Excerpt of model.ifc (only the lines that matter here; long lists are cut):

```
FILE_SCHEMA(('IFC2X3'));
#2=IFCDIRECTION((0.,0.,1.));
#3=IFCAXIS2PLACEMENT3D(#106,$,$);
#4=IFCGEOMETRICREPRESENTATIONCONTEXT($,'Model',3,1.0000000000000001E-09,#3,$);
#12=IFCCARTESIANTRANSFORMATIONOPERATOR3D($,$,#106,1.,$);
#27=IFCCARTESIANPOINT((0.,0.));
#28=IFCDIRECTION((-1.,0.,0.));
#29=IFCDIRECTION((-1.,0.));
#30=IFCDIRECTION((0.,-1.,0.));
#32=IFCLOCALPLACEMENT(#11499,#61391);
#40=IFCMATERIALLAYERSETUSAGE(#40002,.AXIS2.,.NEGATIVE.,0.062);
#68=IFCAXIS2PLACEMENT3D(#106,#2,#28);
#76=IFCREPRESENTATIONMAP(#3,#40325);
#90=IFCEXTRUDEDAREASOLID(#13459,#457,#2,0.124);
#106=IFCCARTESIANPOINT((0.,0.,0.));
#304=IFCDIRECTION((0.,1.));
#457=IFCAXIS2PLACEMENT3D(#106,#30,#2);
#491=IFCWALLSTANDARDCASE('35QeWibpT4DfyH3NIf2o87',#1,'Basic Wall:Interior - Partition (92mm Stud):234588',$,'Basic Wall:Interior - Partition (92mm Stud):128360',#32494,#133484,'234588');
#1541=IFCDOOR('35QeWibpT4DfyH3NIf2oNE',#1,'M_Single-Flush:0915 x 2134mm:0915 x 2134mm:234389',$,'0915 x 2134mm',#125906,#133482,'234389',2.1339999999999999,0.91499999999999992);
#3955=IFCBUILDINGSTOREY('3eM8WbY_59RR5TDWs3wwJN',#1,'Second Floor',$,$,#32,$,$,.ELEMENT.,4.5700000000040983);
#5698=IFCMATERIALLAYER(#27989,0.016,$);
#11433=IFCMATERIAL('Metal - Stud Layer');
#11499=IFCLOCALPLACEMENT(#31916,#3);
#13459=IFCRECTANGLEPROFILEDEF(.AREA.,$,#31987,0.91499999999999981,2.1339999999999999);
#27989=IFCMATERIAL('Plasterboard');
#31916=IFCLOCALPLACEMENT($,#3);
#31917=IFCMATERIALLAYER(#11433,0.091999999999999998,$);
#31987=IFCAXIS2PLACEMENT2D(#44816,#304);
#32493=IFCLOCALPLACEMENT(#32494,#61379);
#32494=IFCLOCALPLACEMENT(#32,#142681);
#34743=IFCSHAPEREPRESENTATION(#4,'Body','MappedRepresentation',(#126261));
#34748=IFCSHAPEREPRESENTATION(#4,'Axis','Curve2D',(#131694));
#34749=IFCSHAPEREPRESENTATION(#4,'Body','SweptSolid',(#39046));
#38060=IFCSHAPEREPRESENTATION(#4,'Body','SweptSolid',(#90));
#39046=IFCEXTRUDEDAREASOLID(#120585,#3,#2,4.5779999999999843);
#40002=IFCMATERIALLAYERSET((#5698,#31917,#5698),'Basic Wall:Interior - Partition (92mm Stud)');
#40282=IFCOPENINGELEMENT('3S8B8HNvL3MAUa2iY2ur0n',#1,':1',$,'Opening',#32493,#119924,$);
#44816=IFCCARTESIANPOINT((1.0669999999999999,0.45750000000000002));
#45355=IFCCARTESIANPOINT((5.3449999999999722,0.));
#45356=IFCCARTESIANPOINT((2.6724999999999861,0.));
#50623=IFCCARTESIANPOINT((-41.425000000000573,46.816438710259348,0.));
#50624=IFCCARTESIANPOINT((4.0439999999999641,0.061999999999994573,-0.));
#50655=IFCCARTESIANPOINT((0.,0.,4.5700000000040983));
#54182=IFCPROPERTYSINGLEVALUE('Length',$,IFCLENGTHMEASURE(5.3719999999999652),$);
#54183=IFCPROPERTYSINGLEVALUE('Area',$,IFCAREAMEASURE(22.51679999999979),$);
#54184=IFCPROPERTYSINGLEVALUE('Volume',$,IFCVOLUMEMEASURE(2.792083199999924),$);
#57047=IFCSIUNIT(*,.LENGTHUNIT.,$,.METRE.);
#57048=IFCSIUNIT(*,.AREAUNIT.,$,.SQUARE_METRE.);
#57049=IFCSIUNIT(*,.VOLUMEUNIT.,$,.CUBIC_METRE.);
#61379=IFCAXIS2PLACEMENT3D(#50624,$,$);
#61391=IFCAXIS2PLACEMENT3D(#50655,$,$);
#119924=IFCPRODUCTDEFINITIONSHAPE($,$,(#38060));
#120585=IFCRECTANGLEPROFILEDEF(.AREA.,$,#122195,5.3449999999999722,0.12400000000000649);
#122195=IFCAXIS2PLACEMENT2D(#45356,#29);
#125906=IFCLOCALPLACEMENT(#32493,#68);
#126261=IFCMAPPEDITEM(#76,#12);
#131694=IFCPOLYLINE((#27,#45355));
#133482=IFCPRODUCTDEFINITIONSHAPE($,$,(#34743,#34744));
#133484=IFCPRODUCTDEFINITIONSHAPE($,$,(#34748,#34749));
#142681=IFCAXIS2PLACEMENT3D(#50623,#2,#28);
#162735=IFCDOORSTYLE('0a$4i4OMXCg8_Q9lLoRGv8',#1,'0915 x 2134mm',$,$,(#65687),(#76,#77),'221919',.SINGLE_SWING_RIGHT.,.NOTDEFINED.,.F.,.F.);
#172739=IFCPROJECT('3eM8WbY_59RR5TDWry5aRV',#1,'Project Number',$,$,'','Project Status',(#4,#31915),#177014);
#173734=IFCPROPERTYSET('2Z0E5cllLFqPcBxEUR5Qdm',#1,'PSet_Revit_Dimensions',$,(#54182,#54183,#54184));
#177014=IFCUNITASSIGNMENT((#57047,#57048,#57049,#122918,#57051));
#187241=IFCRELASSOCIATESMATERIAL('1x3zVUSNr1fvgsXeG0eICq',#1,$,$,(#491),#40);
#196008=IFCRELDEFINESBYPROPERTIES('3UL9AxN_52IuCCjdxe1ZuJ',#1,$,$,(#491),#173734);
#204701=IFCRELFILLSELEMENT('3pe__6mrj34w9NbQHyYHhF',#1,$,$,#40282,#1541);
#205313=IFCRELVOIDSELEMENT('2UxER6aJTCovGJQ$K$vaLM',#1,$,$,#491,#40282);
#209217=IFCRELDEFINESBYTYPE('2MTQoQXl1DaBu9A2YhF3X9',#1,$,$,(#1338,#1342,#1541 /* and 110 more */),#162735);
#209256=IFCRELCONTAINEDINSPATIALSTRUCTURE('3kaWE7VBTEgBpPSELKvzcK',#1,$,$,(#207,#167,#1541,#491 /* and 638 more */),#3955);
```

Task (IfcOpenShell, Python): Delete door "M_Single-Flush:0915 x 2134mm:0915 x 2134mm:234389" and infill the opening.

```python
import ifcopenshell
import ifcopenshell.api.feature
import ifcopenshell.api.pset
import ifcopenshell.api.root
import ifcopenshell.geom
import ifcopenshell.util.element
import ifcopenshell.util.shape
import ifcopenshell.util.unit

model = ifcopenshell.open("model.ifc")
area_scale = ifcopenshell.util.unit.calculate_unit_scale(model, "AREAUNIT")
volume_scale = ifcopenshell.util.unit.calculate_unit_scale(model, "VOLUMEUNIT")
settings = ifcopenshell.geom.settings()


def volume(element):
    """Net volume in cubic metres, openings subtracted."""
    shape = ifcopenshell.geom.create_shape(settings, element)
    return ifcopenshell.util.shape.get_volume(shape.geometry)


door = model.by_guid("35QeWibpT4DfyH3NIf2oNE")
opening = door.FillsVoids[0].RelatingOpeningElement
wall = opening.VoidsElements[0].RelatingBuildingElement
before = volume(wall)

ifcopenshell.api.root.remove_product(model, product=door)
ifcopenshell.api.feature.remove_feature(model, feature=opening)

after = volume(wall)
thickness = 0.124  # wall thickness in metres

# Update the wall's stored quantities.
pset = model.by_id(ifcopenshell.util.element.get_pset(wall, "PSet_Revit_Dimensions", should_inherit=False)["id"])
ifcopenshell.api.pset.edit_pset(model, pset=pset, properties={
    "Area": model.create_entity("IfcAreaMeasure", after / thickness / area_scale),
    "Volume": model.create_entity("IfcVolumeMeasure", after / volume_scale),
})

print(f"wall volume {before:.3f} -> {after:.3f} m3")

model.write("model_rev.ifc")
```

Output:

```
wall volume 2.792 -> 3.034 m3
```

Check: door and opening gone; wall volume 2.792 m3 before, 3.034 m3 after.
